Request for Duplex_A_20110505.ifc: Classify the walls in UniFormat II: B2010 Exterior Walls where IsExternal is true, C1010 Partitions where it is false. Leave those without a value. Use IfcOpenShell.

First a look at what the model holds.

```python
import ifcopenshell
import ifcopenshell.util.element

model = ifcopenshell.open("Duplex_A_20110505.ifc")
print(model.schema)
print("classifications:", [c.Name for c in model.by_type("IfcClassification")])
values = [ifcopenshell.util.element.get_pset(e, "Pset_WallCommon", "IsExternal") for e in model.by_type("IfcWall")]
for value in (True, False, None):
    print("IsExternal", value, values.count(value))
```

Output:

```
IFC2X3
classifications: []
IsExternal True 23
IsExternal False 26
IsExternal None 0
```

```python
import ifcopenshell
import ifcopenshell.api.classification
import ifcopenshell.util.element

model = ifcopenshell.open("Duplex_A_20110505.ifc")

# IFC2X3 requires Source and Edition and has no link from the project to the system.
system = model.create_entity("IfcClassification", Source="ASTM", Edition="E1557", Name="UniFormat II")

walls = model.by_type("IfcWall")
external = {e: ifcopenshell.util.element.get_pset(e, "Pset_WallCommon", "IsExternal") for e in walls}
for flag, code, name in ((True, "B2010", "Exterior Walls"), (False, "C1010", "Partitions")):
    products = [e for e in walls if external[e] is flag]
    ifcopenshell.api.classification.add_reference(
        model, products=products, classification=system, identification=code, name=name
    )
    print(code, len(products))

model.write("Duplex_A_20110505_rev.ifc")
```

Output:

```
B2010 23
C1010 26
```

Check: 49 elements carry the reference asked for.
